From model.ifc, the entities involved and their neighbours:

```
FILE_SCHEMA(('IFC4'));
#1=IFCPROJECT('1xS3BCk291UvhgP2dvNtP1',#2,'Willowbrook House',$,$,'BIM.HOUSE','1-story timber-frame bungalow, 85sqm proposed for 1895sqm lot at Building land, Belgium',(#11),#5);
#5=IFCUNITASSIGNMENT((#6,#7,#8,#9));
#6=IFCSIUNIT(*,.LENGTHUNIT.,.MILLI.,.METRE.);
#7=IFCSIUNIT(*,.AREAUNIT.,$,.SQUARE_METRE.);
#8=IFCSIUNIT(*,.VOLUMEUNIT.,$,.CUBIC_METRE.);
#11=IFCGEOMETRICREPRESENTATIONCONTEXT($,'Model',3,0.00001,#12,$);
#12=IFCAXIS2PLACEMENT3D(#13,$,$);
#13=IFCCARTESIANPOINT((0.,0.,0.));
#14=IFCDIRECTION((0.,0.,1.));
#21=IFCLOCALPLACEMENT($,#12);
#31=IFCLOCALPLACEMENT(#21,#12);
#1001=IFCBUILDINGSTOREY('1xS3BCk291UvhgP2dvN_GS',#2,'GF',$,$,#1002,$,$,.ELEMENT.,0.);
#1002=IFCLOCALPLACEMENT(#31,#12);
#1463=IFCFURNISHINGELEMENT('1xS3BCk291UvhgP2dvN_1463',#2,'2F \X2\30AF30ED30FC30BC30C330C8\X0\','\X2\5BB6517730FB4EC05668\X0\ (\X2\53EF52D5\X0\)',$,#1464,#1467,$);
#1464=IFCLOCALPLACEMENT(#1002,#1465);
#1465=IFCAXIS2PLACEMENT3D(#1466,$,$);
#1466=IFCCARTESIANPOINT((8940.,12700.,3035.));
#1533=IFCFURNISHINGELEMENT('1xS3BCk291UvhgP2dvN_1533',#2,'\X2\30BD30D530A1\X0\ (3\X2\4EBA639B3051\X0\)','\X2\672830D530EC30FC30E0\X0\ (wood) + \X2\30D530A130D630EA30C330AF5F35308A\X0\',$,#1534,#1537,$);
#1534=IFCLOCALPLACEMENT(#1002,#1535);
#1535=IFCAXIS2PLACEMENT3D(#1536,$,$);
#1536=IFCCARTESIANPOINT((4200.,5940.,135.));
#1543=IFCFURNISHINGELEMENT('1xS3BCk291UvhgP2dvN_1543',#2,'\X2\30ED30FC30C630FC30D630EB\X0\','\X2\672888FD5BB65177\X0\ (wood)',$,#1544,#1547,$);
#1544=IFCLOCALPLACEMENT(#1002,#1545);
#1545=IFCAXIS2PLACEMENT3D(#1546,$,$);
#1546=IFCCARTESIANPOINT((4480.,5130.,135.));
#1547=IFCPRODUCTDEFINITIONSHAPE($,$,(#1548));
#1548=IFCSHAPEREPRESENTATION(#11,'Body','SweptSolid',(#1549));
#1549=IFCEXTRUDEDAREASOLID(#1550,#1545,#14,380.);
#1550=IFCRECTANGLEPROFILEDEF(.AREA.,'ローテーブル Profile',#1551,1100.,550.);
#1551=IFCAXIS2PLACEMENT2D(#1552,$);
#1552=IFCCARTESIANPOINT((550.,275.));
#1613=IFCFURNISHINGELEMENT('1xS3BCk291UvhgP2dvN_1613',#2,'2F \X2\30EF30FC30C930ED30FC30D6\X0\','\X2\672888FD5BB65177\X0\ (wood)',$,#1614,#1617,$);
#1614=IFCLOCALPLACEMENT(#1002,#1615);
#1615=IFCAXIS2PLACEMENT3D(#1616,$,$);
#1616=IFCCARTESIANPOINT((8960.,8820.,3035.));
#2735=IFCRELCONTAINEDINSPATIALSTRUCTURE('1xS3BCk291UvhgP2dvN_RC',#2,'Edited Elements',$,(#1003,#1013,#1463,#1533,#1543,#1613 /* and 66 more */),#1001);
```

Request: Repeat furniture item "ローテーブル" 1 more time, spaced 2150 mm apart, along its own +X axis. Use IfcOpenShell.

```python
import ifcopenshell
import ifcopenshell.api.geometry
import ifcopenshell.api.root
import ifcopenshell.util.element
import ifcopenshell.util.placement
import ifcopenshell.util.unit

model = ifcopenshell.open("model.ifc")
unit_scale = ifcopenshell.util.unit.calculate_unit_scale(model)


def reuse_history(source, copy):
    """copy_class also copies each property set's owner history, people and application; keep the originals."""
    for rel in copy.IsDefinedBy:
        if rel.is_a("IfcRelDefinesByProperties") and (history := rel.RelatingPropertyDefinition.OwnerHistory):
            rel.RelatingPropertyDefinition.OwnerHistory = source.OwnerHistory
            ifcopenshell.util.element.remove_deep2(model, history)


source = model.by_guid("1xS3BCk291UvhgP2dvN_1543")
base = ifcopenshell.util.placement.get_local_placement(source.ObjectPlacement)
step = base[:3, 0] * 2.15 / unit_scale

for i in range(1, 2):
    copy = ifcopenshell.api.root.copy_class(model, product=source)
    copy.Representation = ifcopenshell.util.element.copy_deep(
        model, source.Representation, exclude=["IfcGeometricRepresentationContext", "IfcRepresentationMap"]
    )
    reuse_history(source, copy)
    matrix = base.copy()
    matrix[:3, 3] += i * step
    print("added at", matrix[:3, 3].round(3) + 0.0)
    ifcopenshell.api.geometry.edit_object_placement(model, product=copy, matrix=matrix, is_si=False)

model.write("model_updated.ifc")
```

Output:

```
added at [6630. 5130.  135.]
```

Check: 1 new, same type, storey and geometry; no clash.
